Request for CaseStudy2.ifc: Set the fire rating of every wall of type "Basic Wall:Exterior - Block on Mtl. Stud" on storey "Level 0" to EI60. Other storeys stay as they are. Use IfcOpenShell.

First a look at what the model holds.

```python
import ifcopenshell
import ifcopenshell.util.element

model = ifcopenshell.open("CaseStudy2.ifc")
print(model.schema)
storey = next(s for s in model.by_type("IfcBuildingStorey") if s.Name == "Level 0")
walls = [e for e in ifcopenshell.util.element.get_decomposition(storey) if e.is_a("IfcWall")]
seen = {}
for e in walls:
    element_type = ifcopenshell.util.element.get_type(e)
    key = (element_type.Name if element_type != e and element_type else None, ifcopenshell.util.element.get_pset(e, "Pset_WallCommon", "FireRating"))
    seen[key] = seen.get(key, 0) + 1
for (name, value), count in sorted(seen.items(), key=str):
    print(count, "x", name, "|", value)
```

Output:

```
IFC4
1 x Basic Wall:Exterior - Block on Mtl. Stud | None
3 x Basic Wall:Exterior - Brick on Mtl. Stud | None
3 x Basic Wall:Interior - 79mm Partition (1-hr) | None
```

```python
import ifcopenshell
import ifcopenshell.api.pset
import ifcopenshell.util.element

model = ifcopenshell.open("CaseStudy2.ifc")

storey = next(s for s in model.by_type("IfcBuildingStorey") if s.Name == "Level 0")
walls = [e for e in ifcopenshell.util.element.get_decomposition(storey) if e.is_a("IfcWall")]

count = 0
for e in walls:
    element_type = ifcopenshell.util.element.get_type(e)
    if element_type in (None, e) or element_type.Name != "Basic Wall:Exterior - Block on Mtl. Stud":
        continue
    # add_pset returns the element's existing set when there is one.
    pset = ifcopenshell.api.pset.add_pset(model, product=e, name="Pset_WallCommon")
    ifcopenshell.api.pset.edit_pset(model, pset=pset, properties={"FireRating": "EI60"})
    count += 1

print(count, "walls updated")

model.write("CaseStudy2_rev.ifc")
```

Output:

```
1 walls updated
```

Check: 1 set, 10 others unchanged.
